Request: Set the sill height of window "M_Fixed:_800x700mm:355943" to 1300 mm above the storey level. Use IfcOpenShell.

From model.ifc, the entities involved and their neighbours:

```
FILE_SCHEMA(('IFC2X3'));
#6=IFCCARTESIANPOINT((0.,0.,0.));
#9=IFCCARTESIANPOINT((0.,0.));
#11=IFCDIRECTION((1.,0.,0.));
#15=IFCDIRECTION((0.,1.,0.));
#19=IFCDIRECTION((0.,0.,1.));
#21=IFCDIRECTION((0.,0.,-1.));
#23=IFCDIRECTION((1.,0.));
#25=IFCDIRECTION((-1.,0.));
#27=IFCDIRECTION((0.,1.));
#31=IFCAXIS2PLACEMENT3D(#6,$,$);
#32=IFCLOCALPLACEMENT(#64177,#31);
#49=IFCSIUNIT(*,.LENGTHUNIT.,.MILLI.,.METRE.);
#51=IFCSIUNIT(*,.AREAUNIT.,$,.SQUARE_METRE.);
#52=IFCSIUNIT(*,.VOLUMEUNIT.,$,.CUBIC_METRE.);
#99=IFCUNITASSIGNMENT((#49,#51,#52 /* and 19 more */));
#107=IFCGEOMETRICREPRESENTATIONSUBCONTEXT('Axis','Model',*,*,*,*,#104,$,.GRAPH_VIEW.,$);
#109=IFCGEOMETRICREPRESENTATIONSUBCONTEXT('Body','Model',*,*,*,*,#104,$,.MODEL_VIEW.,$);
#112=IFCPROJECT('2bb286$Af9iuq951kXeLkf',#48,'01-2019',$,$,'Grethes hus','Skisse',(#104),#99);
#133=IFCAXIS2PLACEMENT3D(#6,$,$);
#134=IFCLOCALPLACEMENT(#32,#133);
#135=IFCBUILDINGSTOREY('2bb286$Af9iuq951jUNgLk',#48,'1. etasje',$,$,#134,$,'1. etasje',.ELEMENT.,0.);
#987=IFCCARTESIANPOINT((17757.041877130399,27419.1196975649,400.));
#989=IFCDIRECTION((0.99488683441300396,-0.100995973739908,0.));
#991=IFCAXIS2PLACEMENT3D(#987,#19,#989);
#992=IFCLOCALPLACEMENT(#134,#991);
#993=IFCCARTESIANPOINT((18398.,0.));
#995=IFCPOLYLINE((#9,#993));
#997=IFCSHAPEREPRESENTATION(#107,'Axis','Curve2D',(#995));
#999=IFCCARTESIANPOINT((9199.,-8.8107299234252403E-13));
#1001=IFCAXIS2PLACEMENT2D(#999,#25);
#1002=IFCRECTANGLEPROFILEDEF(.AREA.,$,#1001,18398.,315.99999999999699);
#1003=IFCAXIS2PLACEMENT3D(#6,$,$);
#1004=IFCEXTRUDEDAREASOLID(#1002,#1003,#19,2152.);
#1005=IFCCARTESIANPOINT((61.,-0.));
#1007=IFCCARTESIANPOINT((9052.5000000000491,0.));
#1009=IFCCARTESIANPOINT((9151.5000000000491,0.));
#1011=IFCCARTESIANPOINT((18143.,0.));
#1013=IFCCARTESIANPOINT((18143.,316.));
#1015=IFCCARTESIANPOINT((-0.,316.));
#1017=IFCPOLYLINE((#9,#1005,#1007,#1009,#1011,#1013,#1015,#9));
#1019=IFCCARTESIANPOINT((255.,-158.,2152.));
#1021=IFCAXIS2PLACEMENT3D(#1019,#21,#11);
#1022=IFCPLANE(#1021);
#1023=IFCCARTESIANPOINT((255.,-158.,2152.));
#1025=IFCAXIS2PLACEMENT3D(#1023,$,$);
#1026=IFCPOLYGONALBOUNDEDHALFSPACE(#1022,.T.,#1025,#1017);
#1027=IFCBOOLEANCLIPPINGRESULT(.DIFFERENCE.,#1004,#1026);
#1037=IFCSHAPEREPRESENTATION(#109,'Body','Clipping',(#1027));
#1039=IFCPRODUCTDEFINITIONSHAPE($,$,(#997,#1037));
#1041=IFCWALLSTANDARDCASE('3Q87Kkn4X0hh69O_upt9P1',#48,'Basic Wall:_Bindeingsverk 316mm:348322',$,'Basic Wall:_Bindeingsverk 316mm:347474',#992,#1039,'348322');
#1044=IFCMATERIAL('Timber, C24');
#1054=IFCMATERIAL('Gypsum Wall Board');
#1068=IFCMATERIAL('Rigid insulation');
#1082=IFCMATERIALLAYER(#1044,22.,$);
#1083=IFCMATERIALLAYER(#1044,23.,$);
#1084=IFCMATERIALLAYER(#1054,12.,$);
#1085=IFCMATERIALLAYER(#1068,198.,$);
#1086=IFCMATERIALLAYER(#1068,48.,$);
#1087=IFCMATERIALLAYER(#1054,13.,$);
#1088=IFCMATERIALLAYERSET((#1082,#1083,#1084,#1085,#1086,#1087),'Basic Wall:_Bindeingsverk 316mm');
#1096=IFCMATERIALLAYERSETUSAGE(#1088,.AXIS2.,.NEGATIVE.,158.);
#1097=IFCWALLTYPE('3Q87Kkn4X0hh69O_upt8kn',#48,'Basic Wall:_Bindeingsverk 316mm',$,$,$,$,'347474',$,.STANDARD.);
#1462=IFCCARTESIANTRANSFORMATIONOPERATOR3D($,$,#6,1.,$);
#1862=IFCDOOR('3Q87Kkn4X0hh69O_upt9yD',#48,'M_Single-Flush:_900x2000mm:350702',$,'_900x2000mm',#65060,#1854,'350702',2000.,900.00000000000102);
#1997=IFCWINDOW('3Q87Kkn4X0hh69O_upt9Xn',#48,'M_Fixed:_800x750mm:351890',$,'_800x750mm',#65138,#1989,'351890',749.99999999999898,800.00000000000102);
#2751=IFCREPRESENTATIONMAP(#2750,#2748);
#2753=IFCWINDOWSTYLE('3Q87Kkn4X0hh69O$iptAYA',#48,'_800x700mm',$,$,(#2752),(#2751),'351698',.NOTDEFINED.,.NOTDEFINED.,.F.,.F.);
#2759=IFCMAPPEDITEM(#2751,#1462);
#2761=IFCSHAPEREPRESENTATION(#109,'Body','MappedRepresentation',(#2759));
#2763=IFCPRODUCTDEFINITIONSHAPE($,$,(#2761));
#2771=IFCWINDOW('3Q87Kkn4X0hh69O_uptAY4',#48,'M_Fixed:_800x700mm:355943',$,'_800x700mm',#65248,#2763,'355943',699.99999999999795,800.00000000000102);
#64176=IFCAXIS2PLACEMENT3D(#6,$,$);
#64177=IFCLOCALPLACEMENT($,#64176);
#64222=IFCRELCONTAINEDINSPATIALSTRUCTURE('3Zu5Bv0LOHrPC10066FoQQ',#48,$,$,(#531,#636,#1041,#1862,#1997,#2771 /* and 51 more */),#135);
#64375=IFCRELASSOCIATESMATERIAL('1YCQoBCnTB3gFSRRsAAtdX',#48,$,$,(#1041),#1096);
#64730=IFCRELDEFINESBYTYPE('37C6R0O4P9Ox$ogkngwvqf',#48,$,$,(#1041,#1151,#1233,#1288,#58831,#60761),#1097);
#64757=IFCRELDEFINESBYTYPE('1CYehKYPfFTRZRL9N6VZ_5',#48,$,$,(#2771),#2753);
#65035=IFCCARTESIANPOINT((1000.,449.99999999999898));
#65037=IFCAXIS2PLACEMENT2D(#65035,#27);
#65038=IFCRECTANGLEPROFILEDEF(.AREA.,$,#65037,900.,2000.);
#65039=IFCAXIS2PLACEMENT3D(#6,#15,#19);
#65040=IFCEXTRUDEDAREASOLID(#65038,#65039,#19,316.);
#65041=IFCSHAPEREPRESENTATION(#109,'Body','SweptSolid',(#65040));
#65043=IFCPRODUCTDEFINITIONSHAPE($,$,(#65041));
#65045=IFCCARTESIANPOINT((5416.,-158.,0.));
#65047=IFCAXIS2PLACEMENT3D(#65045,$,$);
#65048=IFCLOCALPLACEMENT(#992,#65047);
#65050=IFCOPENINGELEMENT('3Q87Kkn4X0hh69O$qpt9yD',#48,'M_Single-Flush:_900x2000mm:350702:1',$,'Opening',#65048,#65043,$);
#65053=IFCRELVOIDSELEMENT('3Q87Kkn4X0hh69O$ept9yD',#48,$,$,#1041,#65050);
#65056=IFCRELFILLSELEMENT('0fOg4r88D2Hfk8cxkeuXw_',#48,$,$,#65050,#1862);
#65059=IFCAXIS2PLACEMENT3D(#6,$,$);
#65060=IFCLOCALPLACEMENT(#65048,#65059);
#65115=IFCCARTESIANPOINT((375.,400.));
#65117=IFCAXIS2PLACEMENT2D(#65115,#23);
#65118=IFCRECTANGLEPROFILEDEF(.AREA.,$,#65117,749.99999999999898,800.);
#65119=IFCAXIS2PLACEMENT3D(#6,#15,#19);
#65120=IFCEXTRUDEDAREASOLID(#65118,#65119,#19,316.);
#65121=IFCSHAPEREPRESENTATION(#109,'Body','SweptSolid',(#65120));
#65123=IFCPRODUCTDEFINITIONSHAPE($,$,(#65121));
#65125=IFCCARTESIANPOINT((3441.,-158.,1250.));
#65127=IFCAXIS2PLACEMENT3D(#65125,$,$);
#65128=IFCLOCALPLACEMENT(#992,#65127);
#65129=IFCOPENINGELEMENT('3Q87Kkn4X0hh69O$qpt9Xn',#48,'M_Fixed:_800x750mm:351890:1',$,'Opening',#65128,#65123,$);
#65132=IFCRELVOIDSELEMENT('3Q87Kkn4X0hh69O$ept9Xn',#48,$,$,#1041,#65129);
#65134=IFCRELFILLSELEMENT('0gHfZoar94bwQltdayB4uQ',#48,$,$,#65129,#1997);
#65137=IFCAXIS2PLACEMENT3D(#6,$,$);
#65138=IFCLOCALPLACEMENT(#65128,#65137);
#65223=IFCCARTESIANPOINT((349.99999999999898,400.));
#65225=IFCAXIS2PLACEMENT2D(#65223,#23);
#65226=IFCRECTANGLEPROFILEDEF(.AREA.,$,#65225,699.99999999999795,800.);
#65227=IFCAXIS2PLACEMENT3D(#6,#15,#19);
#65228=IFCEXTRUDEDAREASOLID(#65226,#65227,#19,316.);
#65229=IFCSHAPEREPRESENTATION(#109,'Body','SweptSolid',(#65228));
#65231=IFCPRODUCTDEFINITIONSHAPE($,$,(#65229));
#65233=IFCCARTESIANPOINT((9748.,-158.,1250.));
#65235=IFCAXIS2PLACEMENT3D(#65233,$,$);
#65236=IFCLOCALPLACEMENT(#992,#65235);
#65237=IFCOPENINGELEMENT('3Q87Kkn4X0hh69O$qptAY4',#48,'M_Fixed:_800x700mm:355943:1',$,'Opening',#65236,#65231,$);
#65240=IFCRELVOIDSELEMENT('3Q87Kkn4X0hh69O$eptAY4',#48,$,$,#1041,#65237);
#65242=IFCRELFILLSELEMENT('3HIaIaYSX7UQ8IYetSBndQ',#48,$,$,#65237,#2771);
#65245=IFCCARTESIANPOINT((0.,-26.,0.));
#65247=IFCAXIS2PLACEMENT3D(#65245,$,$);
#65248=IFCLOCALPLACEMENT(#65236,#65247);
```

```python
import numpy as np
import ifcopenshell
import ifcopenshell.api.geometry
import ifcopenshell.geom
import ifcopenshell.util.element
import ifcopenshell.util.placement
import ifcopenshell.util.shape
import ifcopenshell.util.unit

model = ifcopenshell.open("model.ifc")
unit_scale = ifcopenshell.util.unit.calculate_unit_scale(model)

window = model.by_guid("3Q87Kkn4X0hh69O_uptAY4")
opening = window.FillsVoids[0].RelatingOpeningElement
storey = ifcopenshell.util.element.get_container(window, ifc_class="IfcBuildingStorey")
level = ifcopenshell.util.placement.get_local_placement(storey.ObjectPlacement)[2, 3]

# The opening's origin need not be at the sill, so measure its lowest point.
shape = ifcopenshell.geom.create_shape(ifcopenshell.geom.settings(), opening)
bottom = ifcopenshell.util.shape.get_shape_bottom_elevation(shape, shape.geometry) / unit_scale
dz = level + 1.3 / unit_scale - bottom

shift = np.array([0.0, 0.0, dz])
# The window is placed relative to its opening, so it follows when the opening moves.
matrix = ifcopenshell.util.placement.get_local_placement(opening.ObjectPlacement)
matrix[:3, 3] += shift
ifcopenshell.api.geometry.edit_object_placement(
    model, product=opening, matrix=matrix, is_si=False, should_transform_children=True
)

print(f"moved by {dz * unit_scale:+.3f} m")

model.write("model_edited.ifc")
```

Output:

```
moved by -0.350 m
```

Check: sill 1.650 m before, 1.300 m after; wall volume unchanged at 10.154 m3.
